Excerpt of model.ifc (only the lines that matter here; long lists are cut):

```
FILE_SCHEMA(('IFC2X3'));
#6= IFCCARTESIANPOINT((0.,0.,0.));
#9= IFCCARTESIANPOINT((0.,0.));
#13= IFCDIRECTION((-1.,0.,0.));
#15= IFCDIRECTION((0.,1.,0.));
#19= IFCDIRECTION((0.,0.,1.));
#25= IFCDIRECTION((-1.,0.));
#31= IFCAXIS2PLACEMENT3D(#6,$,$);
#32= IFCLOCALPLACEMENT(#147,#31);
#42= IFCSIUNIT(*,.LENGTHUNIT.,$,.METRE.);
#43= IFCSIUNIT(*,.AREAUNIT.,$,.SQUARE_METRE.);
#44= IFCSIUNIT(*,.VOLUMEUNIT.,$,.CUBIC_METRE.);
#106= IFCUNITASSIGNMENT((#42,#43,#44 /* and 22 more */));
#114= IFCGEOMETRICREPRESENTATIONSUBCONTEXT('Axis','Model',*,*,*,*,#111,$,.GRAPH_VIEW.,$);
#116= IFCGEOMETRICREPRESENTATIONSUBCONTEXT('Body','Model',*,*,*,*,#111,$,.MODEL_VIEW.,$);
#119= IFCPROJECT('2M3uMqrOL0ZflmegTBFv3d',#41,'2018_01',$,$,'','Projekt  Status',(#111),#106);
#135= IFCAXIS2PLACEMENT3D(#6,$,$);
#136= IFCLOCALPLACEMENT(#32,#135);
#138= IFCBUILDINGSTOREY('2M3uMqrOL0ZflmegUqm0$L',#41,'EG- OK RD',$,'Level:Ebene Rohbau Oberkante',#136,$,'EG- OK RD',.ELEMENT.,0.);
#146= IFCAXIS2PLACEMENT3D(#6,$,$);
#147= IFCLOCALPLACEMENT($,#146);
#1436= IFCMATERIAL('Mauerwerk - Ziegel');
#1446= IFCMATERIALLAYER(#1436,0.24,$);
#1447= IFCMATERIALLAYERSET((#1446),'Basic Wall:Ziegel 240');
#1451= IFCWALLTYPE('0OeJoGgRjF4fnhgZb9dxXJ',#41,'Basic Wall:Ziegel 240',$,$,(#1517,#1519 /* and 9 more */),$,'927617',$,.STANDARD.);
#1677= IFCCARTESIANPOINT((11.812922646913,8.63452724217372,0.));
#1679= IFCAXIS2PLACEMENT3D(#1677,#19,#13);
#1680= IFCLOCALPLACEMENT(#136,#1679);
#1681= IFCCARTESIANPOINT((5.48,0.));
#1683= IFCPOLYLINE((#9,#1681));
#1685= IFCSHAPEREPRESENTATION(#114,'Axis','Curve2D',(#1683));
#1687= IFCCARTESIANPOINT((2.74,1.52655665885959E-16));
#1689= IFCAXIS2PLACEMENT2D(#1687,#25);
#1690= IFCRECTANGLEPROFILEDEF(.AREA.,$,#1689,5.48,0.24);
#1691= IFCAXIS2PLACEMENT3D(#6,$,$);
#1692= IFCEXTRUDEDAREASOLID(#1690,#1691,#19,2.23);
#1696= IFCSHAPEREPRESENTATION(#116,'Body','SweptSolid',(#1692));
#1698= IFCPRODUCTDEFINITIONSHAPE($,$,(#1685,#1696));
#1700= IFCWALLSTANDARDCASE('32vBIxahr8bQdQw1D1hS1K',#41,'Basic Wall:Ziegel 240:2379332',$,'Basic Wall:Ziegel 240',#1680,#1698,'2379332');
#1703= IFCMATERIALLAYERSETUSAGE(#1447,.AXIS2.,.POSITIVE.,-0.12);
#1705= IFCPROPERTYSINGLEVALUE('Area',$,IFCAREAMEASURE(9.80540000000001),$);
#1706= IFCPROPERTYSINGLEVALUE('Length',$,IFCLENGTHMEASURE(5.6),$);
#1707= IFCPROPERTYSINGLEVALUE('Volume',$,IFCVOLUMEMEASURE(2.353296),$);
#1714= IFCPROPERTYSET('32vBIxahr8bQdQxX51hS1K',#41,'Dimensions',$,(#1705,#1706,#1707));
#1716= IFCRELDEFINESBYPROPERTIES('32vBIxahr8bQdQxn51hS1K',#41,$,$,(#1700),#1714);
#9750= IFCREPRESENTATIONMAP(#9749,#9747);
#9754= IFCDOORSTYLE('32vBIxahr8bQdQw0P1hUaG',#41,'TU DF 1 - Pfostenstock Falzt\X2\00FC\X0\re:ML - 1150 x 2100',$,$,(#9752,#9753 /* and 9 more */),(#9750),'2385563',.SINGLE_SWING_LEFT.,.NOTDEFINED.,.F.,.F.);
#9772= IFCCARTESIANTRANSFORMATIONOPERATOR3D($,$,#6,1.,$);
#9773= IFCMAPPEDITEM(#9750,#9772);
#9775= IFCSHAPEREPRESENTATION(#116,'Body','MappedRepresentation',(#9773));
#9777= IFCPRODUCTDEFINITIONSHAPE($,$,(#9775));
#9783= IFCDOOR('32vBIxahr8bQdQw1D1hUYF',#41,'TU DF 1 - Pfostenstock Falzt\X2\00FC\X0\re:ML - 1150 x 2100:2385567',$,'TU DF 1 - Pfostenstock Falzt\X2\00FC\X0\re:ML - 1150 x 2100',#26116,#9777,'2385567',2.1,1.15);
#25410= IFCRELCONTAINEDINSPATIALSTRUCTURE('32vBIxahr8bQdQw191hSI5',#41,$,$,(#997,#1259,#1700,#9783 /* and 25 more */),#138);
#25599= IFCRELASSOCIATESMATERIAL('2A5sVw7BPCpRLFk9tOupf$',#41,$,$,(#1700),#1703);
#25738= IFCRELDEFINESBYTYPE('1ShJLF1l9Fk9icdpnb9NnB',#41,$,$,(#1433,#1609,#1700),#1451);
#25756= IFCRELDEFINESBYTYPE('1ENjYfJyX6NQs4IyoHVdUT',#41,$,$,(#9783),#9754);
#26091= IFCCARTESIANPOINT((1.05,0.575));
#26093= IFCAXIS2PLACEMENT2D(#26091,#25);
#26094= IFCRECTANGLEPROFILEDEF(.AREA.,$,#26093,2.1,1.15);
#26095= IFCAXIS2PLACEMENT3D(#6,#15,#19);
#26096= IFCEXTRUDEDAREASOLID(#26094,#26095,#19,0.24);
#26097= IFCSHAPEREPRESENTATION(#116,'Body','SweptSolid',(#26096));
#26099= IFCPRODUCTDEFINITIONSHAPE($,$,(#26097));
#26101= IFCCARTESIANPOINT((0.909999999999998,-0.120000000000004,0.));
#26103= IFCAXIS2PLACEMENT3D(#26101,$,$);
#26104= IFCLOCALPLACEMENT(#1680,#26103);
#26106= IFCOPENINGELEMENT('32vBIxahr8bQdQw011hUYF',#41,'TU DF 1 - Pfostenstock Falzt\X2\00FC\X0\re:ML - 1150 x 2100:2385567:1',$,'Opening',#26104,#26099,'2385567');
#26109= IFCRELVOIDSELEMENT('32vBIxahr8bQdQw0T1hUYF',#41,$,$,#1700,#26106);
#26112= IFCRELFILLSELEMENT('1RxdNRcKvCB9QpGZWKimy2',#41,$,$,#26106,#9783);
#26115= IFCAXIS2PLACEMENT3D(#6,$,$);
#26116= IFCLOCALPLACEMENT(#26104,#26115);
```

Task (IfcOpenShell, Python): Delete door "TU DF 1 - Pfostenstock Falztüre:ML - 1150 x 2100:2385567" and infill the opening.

```python
import ifcopenshell
import ifcopenshell.api.feature
import ifcopenshell.api.pset
import ifcopenshell.api.root
import ifcopenshell.geom
import ifcopenshell.util.element
import ifcopenshell.util.shape
import ifcopenshell.util.unit

model = ifcopenshell.open("model.ifc")
area_scale = ifcopenshell.util.unit.calculate_unit_scale(model, "AREAUNIT")
volume_scale = ifcopenshell.util.unit.calculate_unit_scale(model, "VOLUMEUNIT")
settings = ifcopenshell.geom.settings()


def volume(element):
    """Net volume in cubic metres, openings subtracted."""
    shape = ifcopenshell.geom.create_shape(settings, element)
    return ifcopenshell.util.shape.get_volume(shape.geometry)


door = model.by_id(9783)
opening = door.FillsVoids[0].RelatingOpeningElement
wall = opening.VoidsElements[0].RelatingBuildingElement
before = volume(wall)

ifcopenshell.api.root.remove_product(model, product=door)
ifcopenshell.api.feature.remove_feature(model, feature=opening)

after = volume(wall)
thickness = 0.24  # wall thickness in metres

# Update the wall's stored quantities.
pset = model.by_id(ifcopenshell.util.element.get_pset(wall, "Dimensions", should_inherit=False)["id"])
ifcopenshell.api.pset.edit_pset(model, pset=pset, properties={
    "Area": model.create_entity("IfcAreaMeasure", after / thickness / area_scale),
    "Volume": model.create_entity("IfcVolumeMeasure", after / volume_scale),
})

print(f"wall volume {before:.3f} -> {after:.3f} m3")

model.write("model-out.ifc")
```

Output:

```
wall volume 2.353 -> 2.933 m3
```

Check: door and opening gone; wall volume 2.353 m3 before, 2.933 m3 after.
